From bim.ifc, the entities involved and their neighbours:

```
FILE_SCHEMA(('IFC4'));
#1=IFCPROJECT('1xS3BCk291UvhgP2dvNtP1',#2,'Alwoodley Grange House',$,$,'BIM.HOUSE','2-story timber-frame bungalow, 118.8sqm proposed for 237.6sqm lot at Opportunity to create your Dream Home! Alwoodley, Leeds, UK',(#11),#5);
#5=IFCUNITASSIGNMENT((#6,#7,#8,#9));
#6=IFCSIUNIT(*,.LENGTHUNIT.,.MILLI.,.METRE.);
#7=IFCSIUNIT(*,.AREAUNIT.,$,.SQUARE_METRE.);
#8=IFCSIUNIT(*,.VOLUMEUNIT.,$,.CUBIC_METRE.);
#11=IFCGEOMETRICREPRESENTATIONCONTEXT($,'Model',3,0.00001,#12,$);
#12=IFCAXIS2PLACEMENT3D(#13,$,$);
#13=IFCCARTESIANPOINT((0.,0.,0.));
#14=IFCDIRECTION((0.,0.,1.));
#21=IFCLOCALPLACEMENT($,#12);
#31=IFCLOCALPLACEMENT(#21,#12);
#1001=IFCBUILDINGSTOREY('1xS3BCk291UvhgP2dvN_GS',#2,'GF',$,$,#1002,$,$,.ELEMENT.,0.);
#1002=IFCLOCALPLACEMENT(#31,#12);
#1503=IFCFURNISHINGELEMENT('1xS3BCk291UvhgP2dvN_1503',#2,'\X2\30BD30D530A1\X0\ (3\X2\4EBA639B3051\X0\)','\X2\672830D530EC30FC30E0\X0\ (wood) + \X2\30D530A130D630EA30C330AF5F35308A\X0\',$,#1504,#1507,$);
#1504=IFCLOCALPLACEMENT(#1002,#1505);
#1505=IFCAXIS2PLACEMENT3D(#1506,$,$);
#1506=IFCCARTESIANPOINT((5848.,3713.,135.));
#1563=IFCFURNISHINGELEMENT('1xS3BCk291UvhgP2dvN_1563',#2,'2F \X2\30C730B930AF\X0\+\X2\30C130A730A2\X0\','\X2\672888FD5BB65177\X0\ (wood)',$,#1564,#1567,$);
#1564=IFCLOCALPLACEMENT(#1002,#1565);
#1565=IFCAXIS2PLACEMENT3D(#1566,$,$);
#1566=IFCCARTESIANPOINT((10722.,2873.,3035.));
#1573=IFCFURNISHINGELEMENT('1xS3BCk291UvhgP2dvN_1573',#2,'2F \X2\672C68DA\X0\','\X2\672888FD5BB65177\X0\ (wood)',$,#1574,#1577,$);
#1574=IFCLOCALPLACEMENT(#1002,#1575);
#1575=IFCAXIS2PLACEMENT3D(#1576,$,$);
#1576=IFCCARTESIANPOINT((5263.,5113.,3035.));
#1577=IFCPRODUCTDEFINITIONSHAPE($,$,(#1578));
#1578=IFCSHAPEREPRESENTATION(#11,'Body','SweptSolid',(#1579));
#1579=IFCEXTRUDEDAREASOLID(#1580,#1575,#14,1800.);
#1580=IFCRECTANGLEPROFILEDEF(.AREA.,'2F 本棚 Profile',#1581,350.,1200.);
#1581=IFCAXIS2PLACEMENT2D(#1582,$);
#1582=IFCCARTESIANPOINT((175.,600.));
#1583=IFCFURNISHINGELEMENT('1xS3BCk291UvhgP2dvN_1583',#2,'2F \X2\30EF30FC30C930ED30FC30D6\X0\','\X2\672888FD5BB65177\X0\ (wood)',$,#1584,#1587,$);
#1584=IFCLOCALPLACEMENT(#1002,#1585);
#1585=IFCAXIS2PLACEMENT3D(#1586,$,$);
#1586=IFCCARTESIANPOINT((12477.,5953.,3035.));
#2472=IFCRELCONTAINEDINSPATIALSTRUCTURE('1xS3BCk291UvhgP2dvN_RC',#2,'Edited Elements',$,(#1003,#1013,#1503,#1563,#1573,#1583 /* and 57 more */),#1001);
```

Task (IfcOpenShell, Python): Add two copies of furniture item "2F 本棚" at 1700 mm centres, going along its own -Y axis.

```python
import ifcopenshell
import ifcopenshell.api.geometry
import ifcopenshell.api.root
import ifcopenshell.util.element
import ifcopenshell.util.placement
import ifcopenshell.util.unit

model = ifcopenshell.open("bim.ifc")
unit_scale = ifcopenshell.util.unit.calculate_unit_scale(model)


def reuse_history(source, copy):
    """copy_class also copies each property set's owner history, people and application; keep the originals."""
    for rel in copy.IsDefinedBy:
        if rel.is_a("IfcRelDefinesByProperties") and (history := rel.RelatingPropertyDefinition.OwnerHistory):
            rel.RelatingPropertyDefinition.OwnerHistory = source.OwnerHistory
            ifcopenshell.util.element.remove_deep2(model, history)


source = model.by_id(1573)
base = ifcopenshell.util.placement.get_local_placement(source.ObjectPlacement)
step = -base[:3, 1] * 1.7 / unit_scale

for i in range(1, 3):
    copy = ifcopenshell.api.root.copy_class(model, product=source)
    copy.Representation = ifcopenshell.util.element.copy_deep(
        model, source.Representation, exclude=["IfcGeometricRepresentationContext", "IfcRepresentationMap"]
    )
    reuse_history(source, copy)
    matrix = base.copy()
    matrix[:3, 3] += i * step
    print("added at", matrix[:3, 3].round(3) + 0.0)
    ifcopenshell.api.geometry.edit_object_placement(model, product=copy, matrix=matrix, is_si=False)

model.write("bim_v2.ifc")
```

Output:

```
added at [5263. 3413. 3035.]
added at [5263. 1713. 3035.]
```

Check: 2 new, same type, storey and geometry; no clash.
